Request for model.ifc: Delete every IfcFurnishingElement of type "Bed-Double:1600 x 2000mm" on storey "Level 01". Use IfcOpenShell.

First a look at what the model holds.

```python
import ifcopenshell
import ifcopenshell.util.element

model = ifcopenshell.open("model.ifc")
print(model.schema)
storey = next(s for s in model.by_type("IfcBuildingStorey") if s.Name == "Level 01")
furniture = [e for e in ifcopenshell.util.element.get_decomposition(storey) if e.is_a("IfcFurnishingElement")]
seen = {}
for e in furniture:
    element_type = ifcopenshell.util.element.get_type(e)
    name = element_type.Name if element_type not in (None, e) else None
    seen[name] = seen.get(name, 0) + 1
for name, count in sorted(seen.items(), key=str):
    print(count, "x", name)
```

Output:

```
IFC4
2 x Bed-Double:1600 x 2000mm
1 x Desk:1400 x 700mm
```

```python
import ifcopenshell
import ifcopenshell.api.root
import ifcopenshell.util.element

model = ifcopenshell.open("model.ifc")

storey = next(s for s in model.by_type("IfcBuildingStorey") if s.Name == "Level 01")
furniture = [e for e in ifcopenshell.util.element.get_decomposition(storey) if e.is_a("IfcFurnishingElement")]
targets = [e for e in furniture if (t := ifcopenshell.util.element.get_type(e)) not in (None, e) and t.Name == "Bed-Double:1600 x 2000mm"]

for e in targets:
    ifcopenshell.api.root.remove_product(model, product=e)
print(len(targets), "removed")

model.write("model_edited.ifc")
```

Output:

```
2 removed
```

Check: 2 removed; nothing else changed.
